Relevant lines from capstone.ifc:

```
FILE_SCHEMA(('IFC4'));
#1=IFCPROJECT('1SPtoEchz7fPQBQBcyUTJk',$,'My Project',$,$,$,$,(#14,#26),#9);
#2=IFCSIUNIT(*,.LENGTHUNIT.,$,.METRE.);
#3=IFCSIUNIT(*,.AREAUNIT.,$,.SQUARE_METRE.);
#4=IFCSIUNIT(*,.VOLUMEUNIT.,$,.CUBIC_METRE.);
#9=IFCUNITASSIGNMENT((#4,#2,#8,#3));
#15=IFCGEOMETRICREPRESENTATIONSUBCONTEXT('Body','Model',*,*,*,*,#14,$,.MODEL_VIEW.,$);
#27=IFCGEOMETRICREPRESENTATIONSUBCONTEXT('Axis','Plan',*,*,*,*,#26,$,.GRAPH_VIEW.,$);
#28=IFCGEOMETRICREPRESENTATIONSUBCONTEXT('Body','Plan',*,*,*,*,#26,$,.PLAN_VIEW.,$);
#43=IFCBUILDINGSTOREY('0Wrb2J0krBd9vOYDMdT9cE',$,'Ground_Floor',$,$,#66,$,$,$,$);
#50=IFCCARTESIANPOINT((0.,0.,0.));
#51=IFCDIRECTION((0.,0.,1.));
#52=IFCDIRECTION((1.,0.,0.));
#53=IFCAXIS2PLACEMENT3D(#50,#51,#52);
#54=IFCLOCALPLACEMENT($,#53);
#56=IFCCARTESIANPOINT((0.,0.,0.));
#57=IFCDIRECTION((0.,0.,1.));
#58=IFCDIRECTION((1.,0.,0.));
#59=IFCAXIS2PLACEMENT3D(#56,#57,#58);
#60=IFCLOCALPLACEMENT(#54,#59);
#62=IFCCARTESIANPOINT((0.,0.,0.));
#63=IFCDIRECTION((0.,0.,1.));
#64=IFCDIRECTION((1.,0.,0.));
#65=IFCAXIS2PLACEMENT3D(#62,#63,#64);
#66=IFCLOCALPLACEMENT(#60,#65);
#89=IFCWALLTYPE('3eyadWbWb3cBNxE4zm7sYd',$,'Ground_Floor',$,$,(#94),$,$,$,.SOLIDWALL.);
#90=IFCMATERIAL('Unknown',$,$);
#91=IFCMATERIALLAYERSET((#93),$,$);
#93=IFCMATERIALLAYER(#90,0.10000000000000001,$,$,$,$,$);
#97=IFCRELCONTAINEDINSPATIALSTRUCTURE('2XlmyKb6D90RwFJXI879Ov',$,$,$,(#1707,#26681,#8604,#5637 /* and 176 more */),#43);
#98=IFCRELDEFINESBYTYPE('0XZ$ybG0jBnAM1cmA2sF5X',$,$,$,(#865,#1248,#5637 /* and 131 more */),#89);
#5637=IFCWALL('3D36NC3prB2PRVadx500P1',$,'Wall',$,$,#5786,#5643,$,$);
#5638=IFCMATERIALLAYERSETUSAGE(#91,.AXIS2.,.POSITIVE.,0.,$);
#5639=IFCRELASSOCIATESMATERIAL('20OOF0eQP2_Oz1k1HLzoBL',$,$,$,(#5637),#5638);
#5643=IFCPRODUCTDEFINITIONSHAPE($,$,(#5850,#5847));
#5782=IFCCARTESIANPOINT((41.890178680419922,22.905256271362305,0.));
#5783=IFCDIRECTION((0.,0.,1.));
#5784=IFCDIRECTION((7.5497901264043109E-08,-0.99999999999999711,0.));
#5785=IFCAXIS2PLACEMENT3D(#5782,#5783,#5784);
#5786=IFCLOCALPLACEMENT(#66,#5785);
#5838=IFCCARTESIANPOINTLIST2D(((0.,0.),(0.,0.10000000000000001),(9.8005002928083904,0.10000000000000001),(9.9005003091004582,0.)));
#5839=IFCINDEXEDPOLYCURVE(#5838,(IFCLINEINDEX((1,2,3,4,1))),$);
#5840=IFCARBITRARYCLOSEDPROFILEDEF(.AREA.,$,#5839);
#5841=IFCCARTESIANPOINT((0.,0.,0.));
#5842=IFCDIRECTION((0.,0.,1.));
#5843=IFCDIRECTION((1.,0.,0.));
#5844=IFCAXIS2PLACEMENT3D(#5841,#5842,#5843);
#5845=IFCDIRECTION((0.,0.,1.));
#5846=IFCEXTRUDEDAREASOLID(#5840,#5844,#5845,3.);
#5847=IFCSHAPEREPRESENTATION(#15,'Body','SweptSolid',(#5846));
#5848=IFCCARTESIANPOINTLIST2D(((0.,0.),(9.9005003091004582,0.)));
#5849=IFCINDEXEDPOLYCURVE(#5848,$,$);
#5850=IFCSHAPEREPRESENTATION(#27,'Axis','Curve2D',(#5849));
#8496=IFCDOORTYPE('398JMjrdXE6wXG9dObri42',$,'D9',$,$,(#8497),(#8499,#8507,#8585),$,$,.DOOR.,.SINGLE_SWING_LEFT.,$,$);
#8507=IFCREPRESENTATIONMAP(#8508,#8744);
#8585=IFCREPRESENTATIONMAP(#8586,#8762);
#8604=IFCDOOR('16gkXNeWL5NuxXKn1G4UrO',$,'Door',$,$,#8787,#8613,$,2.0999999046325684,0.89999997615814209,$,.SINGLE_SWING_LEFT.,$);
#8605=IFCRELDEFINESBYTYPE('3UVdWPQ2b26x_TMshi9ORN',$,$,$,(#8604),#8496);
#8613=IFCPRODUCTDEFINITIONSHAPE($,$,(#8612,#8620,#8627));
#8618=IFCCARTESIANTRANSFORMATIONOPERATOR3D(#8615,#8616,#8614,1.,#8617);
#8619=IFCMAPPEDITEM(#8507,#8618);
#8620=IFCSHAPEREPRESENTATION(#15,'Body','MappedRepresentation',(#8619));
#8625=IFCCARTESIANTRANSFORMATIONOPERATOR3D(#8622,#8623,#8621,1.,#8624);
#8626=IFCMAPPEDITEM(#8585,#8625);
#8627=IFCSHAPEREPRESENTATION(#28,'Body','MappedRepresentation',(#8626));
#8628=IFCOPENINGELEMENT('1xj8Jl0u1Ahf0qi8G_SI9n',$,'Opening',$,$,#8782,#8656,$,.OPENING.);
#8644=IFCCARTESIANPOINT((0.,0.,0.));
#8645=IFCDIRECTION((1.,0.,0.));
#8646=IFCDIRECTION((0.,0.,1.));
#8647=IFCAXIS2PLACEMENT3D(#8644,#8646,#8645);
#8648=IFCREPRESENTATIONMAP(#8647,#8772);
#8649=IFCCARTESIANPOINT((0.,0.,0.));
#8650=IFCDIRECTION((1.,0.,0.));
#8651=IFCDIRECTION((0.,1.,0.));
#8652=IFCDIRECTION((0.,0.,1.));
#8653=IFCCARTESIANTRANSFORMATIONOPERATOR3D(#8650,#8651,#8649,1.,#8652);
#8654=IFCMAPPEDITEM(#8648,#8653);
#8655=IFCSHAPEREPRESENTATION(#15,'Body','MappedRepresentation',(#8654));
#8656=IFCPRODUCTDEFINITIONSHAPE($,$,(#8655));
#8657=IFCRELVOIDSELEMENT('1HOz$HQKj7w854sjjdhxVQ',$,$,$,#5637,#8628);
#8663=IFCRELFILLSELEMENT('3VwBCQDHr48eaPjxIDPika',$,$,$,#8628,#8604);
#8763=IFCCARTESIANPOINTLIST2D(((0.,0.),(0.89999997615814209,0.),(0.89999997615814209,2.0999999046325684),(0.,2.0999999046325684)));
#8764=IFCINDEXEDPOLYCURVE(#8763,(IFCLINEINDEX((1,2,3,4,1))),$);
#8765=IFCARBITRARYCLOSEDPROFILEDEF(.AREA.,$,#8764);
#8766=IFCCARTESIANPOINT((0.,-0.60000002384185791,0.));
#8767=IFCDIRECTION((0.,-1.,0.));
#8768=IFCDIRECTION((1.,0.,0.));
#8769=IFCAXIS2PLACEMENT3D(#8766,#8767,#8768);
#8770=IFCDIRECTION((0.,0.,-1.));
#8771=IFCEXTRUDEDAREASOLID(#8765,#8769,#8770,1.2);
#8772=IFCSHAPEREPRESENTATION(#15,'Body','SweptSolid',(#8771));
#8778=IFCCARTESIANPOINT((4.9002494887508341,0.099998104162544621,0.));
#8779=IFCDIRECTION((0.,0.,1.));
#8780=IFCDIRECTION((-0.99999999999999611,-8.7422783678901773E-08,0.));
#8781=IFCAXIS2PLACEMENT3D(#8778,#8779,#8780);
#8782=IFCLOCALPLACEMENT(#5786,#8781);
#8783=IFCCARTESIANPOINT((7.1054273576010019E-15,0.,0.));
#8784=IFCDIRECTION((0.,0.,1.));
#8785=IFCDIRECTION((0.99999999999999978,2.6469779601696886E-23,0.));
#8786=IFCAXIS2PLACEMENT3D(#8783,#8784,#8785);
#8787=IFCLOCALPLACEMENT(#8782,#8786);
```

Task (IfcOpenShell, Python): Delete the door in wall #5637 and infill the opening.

```python
import ifcopenshell
import ifcopenshell.api.feature
import ifcopenshell.api.root
import ifcopenshell.geom
import ifcopenshell.util.shape

model = ifcopenshell.open("capstone.ifc")
settings = ifcopenshell.geom.settings()


def volume(element):
    """Net volume in cubic metres, openings subtracted."""
    shape = ifcopenshell.geom.create_shape(settings, element)
    return ifcopenshell.util.shape.get_volume(shape.geometry)


door = model.by_guid("16gkXNeWL5NuxXKn1G4UrO")
opening = door.FillsVoids[0].RelatingOpeningElement
wall = opening.VoidsElements[0].RelatingBuildingElement
before = volume(wall)

ifcopenshell.api.root.remove_product(model, product=door)
ifcopenshell.api.feature.remove_feature(model, feature=opening)

after = volume(wall)

print(f"wall volume {before:.3f} -> {after:.3f} m3")

model.write("capstone_updated.ifc")
```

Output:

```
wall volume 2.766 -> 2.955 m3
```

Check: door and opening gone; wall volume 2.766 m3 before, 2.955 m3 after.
